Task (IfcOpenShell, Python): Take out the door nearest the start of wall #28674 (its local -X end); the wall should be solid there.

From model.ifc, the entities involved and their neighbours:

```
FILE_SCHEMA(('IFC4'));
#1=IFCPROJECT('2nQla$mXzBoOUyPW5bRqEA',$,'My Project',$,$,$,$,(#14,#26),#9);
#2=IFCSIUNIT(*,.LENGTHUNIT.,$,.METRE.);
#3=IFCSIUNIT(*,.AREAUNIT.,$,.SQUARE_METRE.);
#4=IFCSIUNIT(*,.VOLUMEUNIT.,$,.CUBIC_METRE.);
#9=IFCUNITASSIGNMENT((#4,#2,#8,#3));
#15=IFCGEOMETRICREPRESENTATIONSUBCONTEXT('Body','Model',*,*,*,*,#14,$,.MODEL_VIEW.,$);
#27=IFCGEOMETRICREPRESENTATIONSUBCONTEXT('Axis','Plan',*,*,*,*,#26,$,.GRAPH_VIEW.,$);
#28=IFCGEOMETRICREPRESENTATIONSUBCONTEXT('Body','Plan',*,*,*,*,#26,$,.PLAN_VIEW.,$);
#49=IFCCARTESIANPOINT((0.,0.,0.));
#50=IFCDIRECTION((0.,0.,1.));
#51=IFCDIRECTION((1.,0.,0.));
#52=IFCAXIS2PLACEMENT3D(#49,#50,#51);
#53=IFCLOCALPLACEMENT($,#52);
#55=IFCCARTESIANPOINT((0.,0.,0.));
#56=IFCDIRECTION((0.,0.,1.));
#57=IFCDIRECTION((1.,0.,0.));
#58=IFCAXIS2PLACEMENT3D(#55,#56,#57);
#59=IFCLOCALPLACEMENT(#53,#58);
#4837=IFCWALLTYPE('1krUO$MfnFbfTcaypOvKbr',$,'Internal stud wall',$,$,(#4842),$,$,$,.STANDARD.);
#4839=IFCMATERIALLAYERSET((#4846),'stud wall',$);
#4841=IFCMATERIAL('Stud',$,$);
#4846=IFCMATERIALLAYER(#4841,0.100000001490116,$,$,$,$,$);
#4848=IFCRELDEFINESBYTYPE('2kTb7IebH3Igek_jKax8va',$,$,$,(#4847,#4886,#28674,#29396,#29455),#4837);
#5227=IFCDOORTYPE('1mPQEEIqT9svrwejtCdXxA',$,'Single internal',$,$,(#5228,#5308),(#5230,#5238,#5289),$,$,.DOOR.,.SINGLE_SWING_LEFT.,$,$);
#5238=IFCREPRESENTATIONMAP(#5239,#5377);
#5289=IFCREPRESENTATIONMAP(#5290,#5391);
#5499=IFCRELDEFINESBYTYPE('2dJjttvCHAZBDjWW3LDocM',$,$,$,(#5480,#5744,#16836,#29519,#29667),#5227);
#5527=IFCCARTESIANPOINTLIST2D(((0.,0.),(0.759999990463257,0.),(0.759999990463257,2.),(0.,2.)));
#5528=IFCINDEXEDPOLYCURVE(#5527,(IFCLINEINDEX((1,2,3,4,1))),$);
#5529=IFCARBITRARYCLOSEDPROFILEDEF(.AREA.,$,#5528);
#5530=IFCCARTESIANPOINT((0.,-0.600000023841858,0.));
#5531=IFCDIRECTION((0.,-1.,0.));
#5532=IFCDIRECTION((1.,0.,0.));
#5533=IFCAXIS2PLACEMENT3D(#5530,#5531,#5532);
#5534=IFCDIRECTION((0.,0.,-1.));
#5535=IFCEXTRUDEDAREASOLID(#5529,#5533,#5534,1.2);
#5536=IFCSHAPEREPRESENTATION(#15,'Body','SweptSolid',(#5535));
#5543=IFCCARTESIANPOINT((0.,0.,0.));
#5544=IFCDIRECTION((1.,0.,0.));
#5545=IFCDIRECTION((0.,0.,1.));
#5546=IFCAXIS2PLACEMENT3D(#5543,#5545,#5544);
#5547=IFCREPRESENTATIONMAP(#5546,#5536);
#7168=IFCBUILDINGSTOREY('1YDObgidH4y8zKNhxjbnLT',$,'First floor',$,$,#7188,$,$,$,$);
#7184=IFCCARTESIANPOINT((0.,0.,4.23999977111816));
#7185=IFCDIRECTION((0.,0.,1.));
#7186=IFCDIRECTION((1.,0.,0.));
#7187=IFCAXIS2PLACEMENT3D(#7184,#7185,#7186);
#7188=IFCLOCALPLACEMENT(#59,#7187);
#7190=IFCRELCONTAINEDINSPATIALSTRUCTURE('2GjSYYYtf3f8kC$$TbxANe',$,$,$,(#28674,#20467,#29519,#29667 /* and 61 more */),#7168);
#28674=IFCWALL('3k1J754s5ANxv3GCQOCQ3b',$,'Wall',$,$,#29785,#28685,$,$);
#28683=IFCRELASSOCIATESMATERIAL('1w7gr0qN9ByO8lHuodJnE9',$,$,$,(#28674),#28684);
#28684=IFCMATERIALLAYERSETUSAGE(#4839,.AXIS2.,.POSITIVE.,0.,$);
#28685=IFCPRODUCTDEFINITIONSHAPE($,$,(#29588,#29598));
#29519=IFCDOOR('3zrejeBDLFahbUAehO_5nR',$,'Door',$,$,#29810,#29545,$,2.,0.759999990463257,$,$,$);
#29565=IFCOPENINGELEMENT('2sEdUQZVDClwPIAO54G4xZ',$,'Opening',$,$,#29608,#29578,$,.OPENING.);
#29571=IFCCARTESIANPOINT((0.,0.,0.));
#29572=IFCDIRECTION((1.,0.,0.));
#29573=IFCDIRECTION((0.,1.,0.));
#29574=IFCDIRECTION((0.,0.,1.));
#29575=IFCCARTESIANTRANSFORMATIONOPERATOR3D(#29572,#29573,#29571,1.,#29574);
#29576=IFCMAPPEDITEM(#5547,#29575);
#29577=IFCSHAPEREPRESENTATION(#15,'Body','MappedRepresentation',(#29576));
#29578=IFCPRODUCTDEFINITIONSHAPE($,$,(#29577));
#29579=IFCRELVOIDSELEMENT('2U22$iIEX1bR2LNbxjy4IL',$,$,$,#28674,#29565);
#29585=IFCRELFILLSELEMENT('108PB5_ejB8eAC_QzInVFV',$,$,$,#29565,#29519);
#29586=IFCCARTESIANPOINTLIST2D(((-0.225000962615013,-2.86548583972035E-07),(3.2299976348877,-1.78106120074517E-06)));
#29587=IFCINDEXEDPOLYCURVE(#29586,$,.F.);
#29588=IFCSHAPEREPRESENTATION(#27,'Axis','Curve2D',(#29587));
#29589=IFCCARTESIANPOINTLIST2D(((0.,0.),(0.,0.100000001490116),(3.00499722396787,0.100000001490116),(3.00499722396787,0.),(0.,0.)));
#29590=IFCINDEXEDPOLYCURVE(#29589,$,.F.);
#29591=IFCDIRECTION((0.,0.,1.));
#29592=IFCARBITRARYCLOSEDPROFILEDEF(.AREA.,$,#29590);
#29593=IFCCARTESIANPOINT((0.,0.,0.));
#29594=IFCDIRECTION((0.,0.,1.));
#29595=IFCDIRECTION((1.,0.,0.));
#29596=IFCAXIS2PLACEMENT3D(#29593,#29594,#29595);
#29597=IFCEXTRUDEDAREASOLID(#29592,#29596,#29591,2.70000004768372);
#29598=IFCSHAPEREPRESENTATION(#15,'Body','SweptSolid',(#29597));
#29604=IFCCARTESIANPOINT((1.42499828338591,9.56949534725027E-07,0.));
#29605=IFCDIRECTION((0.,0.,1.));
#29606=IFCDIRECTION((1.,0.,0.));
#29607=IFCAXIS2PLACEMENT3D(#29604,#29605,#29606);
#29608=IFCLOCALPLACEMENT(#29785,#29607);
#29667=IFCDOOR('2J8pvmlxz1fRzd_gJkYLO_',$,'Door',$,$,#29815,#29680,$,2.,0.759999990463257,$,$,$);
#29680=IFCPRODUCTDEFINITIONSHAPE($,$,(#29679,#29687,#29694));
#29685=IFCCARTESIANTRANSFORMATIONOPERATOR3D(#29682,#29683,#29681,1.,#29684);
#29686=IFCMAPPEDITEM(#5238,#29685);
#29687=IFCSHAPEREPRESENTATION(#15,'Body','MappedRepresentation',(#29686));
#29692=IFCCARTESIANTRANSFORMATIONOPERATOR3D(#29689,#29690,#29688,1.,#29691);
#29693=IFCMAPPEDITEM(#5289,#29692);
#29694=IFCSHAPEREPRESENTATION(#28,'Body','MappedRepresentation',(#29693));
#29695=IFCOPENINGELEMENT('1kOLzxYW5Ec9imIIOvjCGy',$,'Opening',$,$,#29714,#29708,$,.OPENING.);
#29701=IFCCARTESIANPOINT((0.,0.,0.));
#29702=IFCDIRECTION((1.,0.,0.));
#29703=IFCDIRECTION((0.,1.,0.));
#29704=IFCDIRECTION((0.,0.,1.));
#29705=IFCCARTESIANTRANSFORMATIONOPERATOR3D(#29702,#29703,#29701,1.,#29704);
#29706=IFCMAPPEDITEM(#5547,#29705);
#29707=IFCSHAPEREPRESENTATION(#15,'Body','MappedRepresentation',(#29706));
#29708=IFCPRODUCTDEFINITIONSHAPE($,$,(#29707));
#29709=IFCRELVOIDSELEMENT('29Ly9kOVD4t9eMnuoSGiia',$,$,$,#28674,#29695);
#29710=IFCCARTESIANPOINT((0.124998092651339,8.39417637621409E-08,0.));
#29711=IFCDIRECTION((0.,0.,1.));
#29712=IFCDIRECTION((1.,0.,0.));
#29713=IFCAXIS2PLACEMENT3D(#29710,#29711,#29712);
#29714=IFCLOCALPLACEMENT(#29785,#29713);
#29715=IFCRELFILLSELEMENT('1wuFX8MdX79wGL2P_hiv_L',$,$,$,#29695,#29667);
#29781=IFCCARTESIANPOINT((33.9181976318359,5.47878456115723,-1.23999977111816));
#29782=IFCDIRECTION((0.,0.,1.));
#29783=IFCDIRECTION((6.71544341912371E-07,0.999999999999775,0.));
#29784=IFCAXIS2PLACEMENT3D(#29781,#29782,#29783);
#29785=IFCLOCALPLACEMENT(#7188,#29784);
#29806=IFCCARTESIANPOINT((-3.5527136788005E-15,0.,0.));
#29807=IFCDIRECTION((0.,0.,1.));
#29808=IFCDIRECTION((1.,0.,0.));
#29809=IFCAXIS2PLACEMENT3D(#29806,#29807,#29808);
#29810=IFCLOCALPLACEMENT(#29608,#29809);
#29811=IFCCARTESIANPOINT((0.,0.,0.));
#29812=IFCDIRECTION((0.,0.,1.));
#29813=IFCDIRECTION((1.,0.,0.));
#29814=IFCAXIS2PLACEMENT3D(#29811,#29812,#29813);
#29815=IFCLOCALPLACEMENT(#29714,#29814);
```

```python
import ifcopenshell
import ifcopenshell.api.feature
import ifcopenshell.api.root
import ifcopenshell.geom
import ifcopenshell.util.shape

model = ifcopenshell.open("model.ifc")
settings = ifcopenshell.geom.settings()


def volume(element):
    """Net volume in cubic metres, openings subtracted."""
    shape = ifcopenshell.geom.create_shape(settings, element)
    return ifcopenshell.util.shape.get_volume(shape.geometry)


door = model.by_guid("2J8pvmlxz1fRzd_gJkYLO_")
opening = door.FillsVoids[0].RelatingOpeningElement
wall = opening.VoidsElements[0].RelatingBuildingElement
before = volume(wall)

ifcopenshell.api.root.remove_product(model, product=door)
ifcopenshell.api.feature.remove_feature(model, feature=opening)

after = volume(wall)

print(f"wall volume {before:.3f} -> {after:.3f} m3")

model.write("model-out.ifc")
```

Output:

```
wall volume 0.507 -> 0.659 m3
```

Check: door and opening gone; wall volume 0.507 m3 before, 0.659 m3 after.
